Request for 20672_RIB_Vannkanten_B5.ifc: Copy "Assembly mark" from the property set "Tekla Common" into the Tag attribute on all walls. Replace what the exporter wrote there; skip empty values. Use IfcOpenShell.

First a look at what the model holds.

```python
import ifcopenshell
import ifcopenshell.util.element

model = ifcopenshell.open("20672_RIB_Vannkanten_B5.ifc")
print(model.schema)
walls = model.by_type("IfcWall")
print(len(walls), "walls")
for e in walls[:8]:
    source = ifcopenshell.util.element.get_pset(e, "Tekla Common", "Assembly mark")
    target = e.Tag
    print(e.id(), repr(source), repr(target), sep=" | ")
```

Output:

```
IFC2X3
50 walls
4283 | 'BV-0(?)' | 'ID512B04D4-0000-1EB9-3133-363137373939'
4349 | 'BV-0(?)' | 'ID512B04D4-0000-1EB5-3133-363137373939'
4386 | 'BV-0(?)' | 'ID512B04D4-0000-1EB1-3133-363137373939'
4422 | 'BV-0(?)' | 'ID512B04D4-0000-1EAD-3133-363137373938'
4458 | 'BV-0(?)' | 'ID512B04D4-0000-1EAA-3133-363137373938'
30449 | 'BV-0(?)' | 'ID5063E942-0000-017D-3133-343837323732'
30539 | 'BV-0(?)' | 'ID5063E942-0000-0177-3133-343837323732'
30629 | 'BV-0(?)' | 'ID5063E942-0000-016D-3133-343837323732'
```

```python
import ifcopenshell
import ifcopenshell.util.element

model = ifcopenshell.open("20672_RIB_Vannkanten_B5.ifc")

count = 0
for e in model.by_type("IfcWall"):
    value = ifcopenshell.util.element.get_pset(e, "Tekla Common", "Assembly mark")
    current = e.Tag
    if not value or not value.strip() or current == value:
        continue
    e.Tag = value
    count += 1

print(count, "walls updated")

model.write("20672_RIB_Vannkanten_B5_v2.ifc")
```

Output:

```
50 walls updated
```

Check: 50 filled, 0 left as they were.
